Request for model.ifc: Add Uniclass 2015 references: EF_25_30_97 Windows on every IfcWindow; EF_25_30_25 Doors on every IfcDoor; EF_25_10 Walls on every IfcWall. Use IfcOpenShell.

First a look at what the model holds.

```python
import ifcopenshell

model = ifcopenshell.open("model.ifc")
print(model.schema)
print("classifications:", [c.Name for c in model.by_type("IfcClassification")])
for ifc_class in ("IfcDoor", "IfcRoof", "IfcStair", "IfcWall", "IfcWindow"):
    print(ifc_class, len(model.by_type(ifc_class)))
```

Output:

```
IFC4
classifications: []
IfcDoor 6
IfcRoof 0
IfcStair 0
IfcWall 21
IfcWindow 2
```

```python
import ifcopenshell
import ifcopenshell.api.classification

model = ifcopenshell.open("model.ifc")

system = ifcopenshell.api.classification.add_classification(model, classification="Uniclass 2015")

codes = {
    "IfcWindow": ("EF_25_30_97", "Windows"),
    "IfcDoor": ("EF_25_30_25", "Doors"),
    "IfcWall": ("EF_25_10", "Walls"),
}
for ifc_class, (code, name) in codes.items():
    products = model.by_type(ifc_class)
    ifcopenshell.api.classification.add_reference(
        model, products=products, classification=system, identification=code, name=name
    )
    print(code, len(products))

model.write("model_rev.ifc")
```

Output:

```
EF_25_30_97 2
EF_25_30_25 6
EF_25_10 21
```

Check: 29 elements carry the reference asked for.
